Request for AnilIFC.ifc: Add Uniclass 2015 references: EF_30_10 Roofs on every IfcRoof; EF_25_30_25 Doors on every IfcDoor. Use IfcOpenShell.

First a look at what the model holds.

```python
import ifcopenshell

model = ifcopenshell.open("AnilIFC.ifc")
print(model.schema)
print("classifications:", [c.Name for c in model.by_type("IfcClassification")])
for ifc_class in ("IfcDoor", "IfcRoof", "IfcStair", "IfcWall", "IfcWindow"):
    print(ifc_class, len(model.by_type(ifc_class)))
```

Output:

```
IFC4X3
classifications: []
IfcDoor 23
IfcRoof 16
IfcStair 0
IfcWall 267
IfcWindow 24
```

```python
import ifcopenshell
import ifcopenshell.api.classification

model = ifcopenshell.open("AnilIFC.ifc")

system = ifcopenshell.api.classification.add_classification(model, classification="Uniclass 2015")

codes = {
    "IfcRoof": ("EF_30_10", "Roofs"),
    "IfcDoor": ("EF_25_30_25", "Doors"),
}
for ifc_class, (code, name) in codes.items():
    products = model.by_type(ifc_class)
    ifcopenshell.api.classification.add_reference(
        model, products=products, classification=system, identification=code, name=name
    )
    print(code, len(products))

model.write("AnilIFC_rev.ifc")
```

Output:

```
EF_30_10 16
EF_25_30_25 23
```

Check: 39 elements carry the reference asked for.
